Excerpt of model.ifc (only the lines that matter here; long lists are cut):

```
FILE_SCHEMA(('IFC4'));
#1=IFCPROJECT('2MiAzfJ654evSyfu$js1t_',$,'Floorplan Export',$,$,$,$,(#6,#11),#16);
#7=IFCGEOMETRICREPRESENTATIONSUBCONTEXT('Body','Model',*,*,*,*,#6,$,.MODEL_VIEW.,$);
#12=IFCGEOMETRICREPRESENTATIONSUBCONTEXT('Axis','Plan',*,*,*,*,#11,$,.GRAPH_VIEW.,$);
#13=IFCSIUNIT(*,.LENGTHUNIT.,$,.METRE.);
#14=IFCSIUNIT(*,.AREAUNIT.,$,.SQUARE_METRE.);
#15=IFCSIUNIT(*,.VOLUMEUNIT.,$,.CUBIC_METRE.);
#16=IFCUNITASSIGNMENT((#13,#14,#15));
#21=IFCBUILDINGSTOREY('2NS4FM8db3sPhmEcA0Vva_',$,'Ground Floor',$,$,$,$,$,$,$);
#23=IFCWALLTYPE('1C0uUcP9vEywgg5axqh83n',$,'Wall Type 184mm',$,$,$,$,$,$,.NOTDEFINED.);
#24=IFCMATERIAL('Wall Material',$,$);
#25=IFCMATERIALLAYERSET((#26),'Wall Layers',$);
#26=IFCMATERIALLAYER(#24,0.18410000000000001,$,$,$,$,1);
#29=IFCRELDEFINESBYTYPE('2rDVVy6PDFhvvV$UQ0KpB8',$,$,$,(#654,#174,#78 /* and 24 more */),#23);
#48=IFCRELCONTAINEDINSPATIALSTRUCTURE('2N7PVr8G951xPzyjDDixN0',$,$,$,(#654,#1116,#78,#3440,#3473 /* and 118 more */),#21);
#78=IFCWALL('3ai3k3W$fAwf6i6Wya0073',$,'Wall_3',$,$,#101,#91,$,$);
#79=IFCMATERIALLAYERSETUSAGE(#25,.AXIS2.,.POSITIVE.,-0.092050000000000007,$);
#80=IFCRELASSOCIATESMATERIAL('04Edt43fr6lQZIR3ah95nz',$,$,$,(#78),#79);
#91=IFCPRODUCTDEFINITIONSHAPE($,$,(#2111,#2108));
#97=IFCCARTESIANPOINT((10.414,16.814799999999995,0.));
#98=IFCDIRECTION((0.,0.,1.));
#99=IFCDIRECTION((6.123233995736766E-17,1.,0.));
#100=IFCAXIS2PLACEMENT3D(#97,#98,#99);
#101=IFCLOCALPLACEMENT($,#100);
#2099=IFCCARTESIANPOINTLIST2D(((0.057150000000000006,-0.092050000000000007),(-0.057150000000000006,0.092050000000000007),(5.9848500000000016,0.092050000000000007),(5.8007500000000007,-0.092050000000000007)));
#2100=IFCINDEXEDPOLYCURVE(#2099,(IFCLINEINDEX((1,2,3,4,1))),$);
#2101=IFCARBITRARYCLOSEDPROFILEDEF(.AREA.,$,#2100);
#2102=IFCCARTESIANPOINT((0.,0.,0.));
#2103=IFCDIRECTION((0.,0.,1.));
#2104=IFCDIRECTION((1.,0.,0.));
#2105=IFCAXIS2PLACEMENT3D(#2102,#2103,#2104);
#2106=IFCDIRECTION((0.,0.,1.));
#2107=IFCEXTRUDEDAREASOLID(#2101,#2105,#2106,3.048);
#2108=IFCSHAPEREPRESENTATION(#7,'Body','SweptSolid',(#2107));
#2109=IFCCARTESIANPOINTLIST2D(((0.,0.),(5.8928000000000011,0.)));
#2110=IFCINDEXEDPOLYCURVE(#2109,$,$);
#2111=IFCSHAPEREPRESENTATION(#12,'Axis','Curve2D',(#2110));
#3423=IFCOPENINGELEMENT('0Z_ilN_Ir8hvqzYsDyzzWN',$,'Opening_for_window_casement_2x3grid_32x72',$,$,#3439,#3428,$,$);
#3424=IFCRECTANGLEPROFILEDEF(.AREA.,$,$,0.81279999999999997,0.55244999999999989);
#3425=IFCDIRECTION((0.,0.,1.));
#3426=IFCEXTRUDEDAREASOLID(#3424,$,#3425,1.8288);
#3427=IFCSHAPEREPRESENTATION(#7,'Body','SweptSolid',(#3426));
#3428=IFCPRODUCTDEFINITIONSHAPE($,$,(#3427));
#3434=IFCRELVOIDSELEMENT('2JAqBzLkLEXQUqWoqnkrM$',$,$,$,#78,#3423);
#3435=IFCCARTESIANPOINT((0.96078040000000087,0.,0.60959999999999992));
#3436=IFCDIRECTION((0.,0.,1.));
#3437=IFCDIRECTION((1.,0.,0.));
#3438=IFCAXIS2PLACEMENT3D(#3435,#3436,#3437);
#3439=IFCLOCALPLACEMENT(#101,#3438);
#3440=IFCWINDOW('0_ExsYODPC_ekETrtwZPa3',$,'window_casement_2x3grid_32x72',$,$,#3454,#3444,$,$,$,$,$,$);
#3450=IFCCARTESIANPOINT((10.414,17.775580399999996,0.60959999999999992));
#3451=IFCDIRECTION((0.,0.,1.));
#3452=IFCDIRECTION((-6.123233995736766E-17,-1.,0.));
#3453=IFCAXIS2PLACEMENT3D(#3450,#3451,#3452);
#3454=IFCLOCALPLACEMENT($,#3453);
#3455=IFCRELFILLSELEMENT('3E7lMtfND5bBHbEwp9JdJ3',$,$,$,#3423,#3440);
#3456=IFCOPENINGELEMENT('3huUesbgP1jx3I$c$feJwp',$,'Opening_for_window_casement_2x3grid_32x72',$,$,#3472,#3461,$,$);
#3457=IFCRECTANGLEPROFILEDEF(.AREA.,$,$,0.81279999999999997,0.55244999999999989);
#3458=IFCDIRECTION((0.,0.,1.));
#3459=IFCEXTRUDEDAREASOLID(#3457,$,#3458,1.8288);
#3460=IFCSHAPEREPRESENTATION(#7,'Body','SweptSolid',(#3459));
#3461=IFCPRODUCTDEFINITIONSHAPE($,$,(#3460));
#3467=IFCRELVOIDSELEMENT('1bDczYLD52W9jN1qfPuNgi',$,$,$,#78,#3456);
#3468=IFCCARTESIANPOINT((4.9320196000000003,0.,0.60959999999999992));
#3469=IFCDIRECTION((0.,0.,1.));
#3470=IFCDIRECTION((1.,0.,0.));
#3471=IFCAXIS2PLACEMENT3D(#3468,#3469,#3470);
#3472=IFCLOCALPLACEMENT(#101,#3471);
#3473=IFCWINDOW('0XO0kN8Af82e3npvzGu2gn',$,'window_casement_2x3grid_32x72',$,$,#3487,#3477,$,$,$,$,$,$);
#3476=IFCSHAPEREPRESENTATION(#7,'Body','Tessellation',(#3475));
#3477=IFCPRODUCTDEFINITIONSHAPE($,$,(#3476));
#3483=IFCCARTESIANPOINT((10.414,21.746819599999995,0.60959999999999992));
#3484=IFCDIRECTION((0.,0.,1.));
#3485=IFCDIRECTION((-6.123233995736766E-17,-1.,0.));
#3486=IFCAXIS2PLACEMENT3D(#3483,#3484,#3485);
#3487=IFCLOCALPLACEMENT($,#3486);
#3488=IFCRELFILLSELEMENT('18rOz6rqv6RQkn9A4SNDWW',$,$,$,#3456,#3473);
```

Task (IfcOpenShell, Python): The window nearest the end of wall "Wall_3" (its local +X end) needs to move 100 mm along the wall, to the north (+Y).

```python
import ifcopenshell
import ifcopenshell.api.geometry
import ifcopenshell.util.placement
import ifcopenshell.util.unit

model = ifcopenshell.open("model.ifc")
unit_scale = ifcopenshell.util.unit.calculate_unit_scale(model)

window = model.by_guid("0XO0kN8Af82e3npvzGu2gn")
opening = window.FillsVoids[0].RelatingOpeningElement
wall = opening.VoidsElements[0].RelatingBuildingElement

wall_matrix = ifcopenshell.util.placement.get_local_placement(wall.ObjectPlacement)
shift = wall_matrix[:3, 0] * 0.1 / unit_scale
before = ifcopenshell.util.placement.get_local_placement(window.ObjectPlacement)[:3, 3].copy()

# The window is not placed relative to its opening, so move both.
for product in (opening, window):
    matrix = ifcopenshell.util.placement.get_local_placement(product.ObjectPlacement)
    matrix[:3, 3] += shift
    ifcopenshell.api.geometry.edit_object_placement(model, product=product, matrix=matrix, is_si=False)

after = ifcopenshell.util.placement.get_local_placement(window.ObjectPlacement)[:3, 3]
print("window moved by", (after - before).round(3) + 0.0)

model.write("model_updated.ifc")
```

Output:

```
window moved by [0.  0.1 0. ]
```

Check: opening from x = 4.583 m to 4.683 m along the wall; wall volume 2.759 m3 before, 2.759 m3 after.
